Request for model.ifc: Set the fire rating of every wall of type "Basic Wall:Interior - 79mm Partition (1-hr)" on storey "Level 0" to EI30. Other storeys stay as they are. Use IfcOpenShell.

First a look at what the model holds.

```python
import ifcopenshell
import ifcopenshell.util.element

model = ifcopenshell.open("model.ifc")
print(model.schema)
storey = next(s for s in model.by_type("IfcBuildingStorey") if s.Name == "Level 0")
walls = [e for e in ifcopenshell.util.element.get_decomposition(storey) if e.is_a("IfcWall")]
seen = {}
for e in walls:
    element_type = ifcopenshell.util.element.get_type(e)
    key = (element_type.Name if element_type != e and element_type else None, ifcopenshell.util.element.get_pset(e, "Pset_WallCommon", "FireRating"))
    seen[key] = seen.get(key, 0) + 1
for (name, value), count in sorted(seen.items(), key=str):
    print(count, "x", name, "|", value)
```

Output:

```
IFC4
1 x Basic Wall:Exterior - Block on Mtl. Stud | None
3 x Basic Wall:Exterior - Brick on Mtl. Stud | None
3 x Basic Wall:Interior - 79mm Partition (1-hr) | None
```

```python
import ifcopenshell
import ifcopenshell.api.pset
import ifcopenshell.util.element

model = ifcopenshell.open("model.ifc")

storey = next(s for s in model.by_type("IfcBuildingStorey") if s.Name == "Level 0")
walls = [e for e in ifcopenshell.util.element.get_decomposition(storey) if e.is_a("IfcWall")]

count = 0
for e in walls:
    element_type = ifcopenshell.util.element.get_type(e)
    if element_type in (None, e) or element_type.Name != "Basic Wall:Interior - 79mm Partition (1-hr)":
        continue
    # add_pset returns the element's existing set when there is one.
    pset = ifcopenshell.api.pset.add_pset(model, product=e, name="Pset_WallCommon")
    ifcopenshell.api.pset.edit_pset(model, pset=pset, properties={"FireRating": "EI30"})
    count += 1

print(count, "walls updated")

model.write("model_edited.ifc")
```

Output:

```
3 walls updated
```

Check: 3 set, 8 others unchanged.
